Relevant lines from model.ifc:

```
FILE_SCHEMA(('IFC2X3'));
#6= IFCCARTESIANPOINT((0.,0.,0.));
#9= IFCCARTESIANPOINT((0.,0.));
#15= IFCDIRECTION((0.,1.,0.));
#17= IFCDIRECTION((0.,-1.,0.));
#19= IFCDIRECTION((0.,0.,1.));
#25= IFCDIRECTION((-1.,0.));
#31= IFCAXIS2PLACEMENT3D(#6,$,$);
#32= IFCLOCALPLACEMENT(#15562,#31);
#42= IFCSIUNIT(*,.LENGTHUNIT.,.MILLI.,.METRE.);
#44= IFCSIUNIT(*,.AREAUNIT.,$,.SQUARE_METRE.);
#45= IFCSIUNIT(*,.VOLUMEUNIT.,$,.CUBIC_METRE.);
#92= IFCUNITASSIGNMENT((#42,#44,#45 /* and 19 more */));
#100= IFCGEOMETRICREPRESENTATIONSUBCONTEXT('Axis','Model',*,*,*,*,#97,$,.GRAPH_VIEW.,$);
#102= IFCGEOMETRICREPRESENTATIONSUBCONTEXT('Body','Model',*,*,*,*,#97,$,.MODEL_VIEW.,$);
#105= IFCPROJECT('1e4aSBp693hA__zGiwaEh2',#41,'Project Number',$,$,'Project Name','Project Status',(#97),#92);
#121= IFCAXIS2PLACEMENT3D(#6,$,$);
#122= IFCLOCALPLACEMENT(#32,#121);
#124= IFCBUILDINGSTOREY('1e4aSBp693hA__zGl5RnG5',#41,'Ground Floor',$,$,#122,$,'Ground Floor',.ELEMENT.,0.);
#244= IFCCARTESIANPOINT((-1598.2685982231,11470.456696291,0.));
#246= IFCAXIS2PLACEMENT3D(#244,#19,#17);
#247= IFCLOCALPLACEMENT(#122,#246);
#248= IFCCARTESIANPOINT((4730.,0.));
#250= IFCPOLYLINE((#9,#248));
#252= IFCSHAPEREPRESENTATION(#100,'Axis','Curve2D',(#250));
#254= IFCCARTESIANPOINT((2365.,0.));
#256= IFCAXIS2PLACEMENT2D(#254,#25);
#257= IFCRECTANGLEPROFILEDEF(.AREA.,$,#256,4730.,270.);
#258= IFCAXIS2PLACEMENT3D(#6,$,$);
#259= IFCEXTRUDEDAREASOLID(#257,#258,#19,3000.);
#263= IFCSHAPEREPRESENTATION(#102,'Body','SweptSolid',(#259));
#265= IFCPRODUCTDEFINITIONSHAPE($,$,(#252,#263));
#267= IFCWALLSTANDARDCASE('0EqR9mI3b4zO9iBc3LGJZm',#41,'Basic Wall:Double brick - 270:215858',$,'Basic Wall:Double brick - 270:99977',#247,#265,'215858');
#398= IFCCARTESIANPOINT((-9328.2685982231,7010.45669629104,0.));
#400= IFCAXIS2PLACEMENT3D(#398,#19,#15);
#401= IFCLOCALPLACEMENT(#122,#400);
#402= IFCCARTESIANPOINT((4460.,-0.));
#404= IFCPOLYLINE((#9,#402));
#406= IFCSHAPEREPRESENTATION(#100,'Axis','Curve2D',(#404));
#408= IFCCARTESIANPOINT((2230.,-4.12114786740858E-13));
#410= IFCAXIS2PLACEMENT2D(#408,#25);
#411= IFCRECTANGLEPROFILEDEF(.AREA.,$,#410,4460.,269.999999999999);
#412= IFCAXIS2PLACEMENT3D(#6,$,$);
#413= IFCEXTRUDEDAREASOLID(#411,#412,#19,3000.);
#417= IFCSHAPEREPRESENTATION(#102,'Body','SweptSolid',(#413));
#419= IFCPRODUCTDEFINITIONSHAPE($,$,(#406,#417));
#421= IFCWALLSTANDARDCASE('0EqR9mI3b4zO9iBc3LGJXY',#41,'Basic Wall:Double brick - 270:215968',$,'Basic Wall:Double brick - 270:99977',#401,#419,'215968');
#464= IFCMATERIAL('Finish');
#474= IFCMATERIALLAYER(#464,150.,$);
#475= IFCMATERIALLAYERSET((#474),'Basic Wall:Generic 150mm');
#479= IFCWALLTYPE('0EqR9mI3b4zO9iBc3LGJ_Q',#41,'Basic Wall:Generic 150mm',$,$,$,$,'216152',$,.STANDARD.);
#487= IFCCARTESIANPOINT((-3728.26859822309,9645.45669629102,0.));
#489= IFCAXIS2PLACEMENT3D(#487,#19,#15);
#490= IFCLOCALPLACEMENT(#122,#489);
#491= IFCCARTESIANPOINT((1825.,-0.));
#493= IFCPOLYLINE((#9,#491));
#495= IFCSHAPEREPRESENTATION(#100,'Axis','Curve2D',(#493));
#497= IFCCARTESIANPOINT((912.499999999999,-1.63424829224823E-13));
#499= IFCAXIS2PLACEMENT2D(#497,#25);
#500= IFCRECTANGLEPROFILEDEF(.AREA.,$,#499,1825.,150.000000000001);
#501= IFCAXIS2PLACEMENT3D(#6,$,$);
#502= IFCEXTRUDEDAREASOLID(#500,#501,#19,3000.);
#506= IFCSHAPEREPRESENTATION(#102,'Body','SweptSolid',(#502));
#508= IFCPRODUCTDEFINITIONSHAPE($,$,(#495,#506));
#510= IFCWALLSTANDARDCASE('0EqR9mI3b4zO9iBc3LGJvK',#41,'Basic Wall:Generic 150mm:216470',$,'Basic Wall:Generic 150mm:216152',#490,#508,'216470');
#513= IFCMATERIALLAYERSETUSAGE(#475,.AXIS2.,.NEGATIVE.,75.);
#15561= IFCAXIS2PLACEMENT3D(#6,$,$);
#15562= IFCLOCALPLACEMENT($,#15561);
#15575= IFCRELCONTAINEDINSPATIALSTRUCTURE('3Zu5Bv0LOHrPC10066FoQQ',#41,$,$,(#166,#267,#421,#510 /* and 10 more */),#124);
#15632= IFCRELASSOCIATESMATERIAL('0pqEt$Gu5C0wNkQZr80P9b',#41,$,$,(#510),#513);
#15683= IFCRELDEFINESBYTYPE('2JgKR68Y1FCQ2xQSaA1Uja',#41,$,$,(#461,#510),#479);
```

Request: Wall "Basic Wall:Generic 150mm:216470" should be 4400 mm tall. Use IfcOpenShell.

```python
import ifcopenshell
import ifcopenshell.geom
import ifcopenshell.util.representation
import ifcopenshell.util.shape
import ifcopenshell.util.unit

model = ifcopenshell.open("model.ifc")
unit_scale = ifcopenshell.util.unit.calculate_unit_scale(model)
settings = ifcopenshell.geom.settings()


def volume(element):
    """Net volume in cubic metres, openings subtracted."""
    shape = ifcopenshell.geom.create_shape(settings, element)
    return ifcopenshell.util.shape.get_volume(shape.geometry)


wall = model.by_guid("0EqR9mI3b4zO9iBc3LGJvK")
before = volume(wall)

body = ifcopenshell.util.representation.get_representation(wall, "Model", "Body")
solid = body.Items[0]
old_height = solid.Depth
solid.Depth = 4.4 / unit_scale
after = volume(wall)

print(f"height {old_height:g} -> {solid.Depth:g}, volume {before:.3f} -> {after:.3f} m3")

model.write("model-out.ifc")
```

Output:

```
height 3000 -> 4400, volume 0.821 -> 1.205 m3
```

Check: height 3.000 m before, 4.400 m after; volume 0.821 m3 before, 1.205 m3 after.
